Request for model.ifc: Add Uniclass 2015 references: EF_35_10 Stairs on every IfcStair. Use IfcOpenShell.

First a look at what the model holds.

```python
import ifcopenshell

model = ifcopenshell.open("model.ifc")
print(model.schema)
print("classifications:", [c.Name for c in model.by_type("IfcClassification")])
for ifc_class in ("IfcDoor", "IfcRoof", "IfcStair", "IfcWall", "IfcWindow"):
    print(ifc_class, len(model.by_type(ifc_class)))
```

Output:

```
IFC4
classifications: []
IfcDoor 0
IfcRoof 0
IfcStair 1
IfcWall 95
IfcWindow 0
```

```python
import ifcopenshell
import ifcopenshell.api.classification

model = ifcopenshell.open("model.ifc")

system = ifcopenshell.api.classification.add_classification(model, classification="Uniclass 2015")

codes = {
    "IfcStair": ("EF_35_10", "Stairs"),
}
for ifc_class, (code, name) in codes.items():
    products = model.by_type(ifc_class)
    ifcopenshell.api.classification.add_reference(
        model, products=products, classification=system, identification=code, name=name
    )
    print(code, len(products))

model.write("model_updated.ifc")
```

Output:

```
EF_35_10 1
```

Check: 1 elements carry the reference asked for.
